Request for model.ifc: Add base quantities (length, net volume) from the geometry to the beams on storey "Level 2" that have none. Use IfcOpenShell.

First a look at what the model holds.

```python
import ifcopenshell
import ifcopenshell.util.element
import ifcopenshell.util.unit

model = ifcopenshell.open("model.ifc")
print(model.schema)
for unit_type in ("LENGTHUNIT", "AREAUNIT", "VOLUMEUNIT"):
    print(unit_type, ifcopenshell.util.unit.calculate_unit_scale(model, unit_type))
storey = next(s for s in model.by_type("IfcBuildingStorey") if s.Name == "Level 2")
beams = [e for e in ifcopenshell.util.element.get_decomposition(storey) if e.is_a("IfcBeam")]
for e in sorted(beams, key=lambda e: e.id()):
    print(e.id(), e.is_a(), e.Name, list(ifcopenshell.util.element.get_psets(e, qtos_only=True)), sep=" | ")
```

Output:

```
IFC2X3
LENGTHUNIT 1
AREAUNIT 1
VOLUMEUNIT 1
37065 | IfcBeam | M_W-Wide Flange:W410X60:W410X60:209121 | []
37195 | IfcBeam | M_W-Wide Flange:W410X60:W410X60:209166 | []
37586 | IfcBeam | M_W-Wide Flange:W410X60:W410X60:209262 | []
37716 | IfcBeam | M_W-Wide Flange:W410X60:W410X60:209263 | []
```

```python
import ifcopenshell
import ifcopenshell.api.pset
import ifcopenshell.geom
import ifcopenshell.util.element
import ifcopenshell.util.shape
import ifcopenshell.util.unit

model = ifcopenshell.open("model.ifc")
unit_scale = ifcopenshell.util.unit.calculate_unit_scale(model)
volume_scale = ifcopenshell.util.unit.calculate_unit_scale(model, "VOLUMEUNIT")
settings = ifcopenshell.geom.settings()

storey = next(s for s in model.by_type("IfcBuildingStorey") if s.Name == "Level 2")
beams = [e for e in ifcopenshell.util.element.get_decomposition(storey) if e.is_a("IfcBeam")]

for e in sorted(beams, key=lambda e: e.id()):
    if ifcopenshell.util.element.get_psets(e, qtos_only=True, should_inherit=False):
        continue
    # Geometry comes back in metres, in the element's own axes.
    shape = ifcopenshell.geom.create_shape(settings, e)
    values = {
        "Length": ifcopenshell.util.shape.get_max_xyz(shape.geometry) / unit_scale,
        "NetVolume": ifcopenshell.util.shape.get_volume(shape.geometry) / volume_scale,
    }
    qto = ifcopenshell.api.pset.add_qto(model, product=e, name="BaseQuantities")
    ifcopenshell.api.pset.edit_qto(model, qto=qto, properties=values)
    print(e.id(), {k: round(v, 3) for k, v in values.items()})

model.write("model_updated.ifc")
```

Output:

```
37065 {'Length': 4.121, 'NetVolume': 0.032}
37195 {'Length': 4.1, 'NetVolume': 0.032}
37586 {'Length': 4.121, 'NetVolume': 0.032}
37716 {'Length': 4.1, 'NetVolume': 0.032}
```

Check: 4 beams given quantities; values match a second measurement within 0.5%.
